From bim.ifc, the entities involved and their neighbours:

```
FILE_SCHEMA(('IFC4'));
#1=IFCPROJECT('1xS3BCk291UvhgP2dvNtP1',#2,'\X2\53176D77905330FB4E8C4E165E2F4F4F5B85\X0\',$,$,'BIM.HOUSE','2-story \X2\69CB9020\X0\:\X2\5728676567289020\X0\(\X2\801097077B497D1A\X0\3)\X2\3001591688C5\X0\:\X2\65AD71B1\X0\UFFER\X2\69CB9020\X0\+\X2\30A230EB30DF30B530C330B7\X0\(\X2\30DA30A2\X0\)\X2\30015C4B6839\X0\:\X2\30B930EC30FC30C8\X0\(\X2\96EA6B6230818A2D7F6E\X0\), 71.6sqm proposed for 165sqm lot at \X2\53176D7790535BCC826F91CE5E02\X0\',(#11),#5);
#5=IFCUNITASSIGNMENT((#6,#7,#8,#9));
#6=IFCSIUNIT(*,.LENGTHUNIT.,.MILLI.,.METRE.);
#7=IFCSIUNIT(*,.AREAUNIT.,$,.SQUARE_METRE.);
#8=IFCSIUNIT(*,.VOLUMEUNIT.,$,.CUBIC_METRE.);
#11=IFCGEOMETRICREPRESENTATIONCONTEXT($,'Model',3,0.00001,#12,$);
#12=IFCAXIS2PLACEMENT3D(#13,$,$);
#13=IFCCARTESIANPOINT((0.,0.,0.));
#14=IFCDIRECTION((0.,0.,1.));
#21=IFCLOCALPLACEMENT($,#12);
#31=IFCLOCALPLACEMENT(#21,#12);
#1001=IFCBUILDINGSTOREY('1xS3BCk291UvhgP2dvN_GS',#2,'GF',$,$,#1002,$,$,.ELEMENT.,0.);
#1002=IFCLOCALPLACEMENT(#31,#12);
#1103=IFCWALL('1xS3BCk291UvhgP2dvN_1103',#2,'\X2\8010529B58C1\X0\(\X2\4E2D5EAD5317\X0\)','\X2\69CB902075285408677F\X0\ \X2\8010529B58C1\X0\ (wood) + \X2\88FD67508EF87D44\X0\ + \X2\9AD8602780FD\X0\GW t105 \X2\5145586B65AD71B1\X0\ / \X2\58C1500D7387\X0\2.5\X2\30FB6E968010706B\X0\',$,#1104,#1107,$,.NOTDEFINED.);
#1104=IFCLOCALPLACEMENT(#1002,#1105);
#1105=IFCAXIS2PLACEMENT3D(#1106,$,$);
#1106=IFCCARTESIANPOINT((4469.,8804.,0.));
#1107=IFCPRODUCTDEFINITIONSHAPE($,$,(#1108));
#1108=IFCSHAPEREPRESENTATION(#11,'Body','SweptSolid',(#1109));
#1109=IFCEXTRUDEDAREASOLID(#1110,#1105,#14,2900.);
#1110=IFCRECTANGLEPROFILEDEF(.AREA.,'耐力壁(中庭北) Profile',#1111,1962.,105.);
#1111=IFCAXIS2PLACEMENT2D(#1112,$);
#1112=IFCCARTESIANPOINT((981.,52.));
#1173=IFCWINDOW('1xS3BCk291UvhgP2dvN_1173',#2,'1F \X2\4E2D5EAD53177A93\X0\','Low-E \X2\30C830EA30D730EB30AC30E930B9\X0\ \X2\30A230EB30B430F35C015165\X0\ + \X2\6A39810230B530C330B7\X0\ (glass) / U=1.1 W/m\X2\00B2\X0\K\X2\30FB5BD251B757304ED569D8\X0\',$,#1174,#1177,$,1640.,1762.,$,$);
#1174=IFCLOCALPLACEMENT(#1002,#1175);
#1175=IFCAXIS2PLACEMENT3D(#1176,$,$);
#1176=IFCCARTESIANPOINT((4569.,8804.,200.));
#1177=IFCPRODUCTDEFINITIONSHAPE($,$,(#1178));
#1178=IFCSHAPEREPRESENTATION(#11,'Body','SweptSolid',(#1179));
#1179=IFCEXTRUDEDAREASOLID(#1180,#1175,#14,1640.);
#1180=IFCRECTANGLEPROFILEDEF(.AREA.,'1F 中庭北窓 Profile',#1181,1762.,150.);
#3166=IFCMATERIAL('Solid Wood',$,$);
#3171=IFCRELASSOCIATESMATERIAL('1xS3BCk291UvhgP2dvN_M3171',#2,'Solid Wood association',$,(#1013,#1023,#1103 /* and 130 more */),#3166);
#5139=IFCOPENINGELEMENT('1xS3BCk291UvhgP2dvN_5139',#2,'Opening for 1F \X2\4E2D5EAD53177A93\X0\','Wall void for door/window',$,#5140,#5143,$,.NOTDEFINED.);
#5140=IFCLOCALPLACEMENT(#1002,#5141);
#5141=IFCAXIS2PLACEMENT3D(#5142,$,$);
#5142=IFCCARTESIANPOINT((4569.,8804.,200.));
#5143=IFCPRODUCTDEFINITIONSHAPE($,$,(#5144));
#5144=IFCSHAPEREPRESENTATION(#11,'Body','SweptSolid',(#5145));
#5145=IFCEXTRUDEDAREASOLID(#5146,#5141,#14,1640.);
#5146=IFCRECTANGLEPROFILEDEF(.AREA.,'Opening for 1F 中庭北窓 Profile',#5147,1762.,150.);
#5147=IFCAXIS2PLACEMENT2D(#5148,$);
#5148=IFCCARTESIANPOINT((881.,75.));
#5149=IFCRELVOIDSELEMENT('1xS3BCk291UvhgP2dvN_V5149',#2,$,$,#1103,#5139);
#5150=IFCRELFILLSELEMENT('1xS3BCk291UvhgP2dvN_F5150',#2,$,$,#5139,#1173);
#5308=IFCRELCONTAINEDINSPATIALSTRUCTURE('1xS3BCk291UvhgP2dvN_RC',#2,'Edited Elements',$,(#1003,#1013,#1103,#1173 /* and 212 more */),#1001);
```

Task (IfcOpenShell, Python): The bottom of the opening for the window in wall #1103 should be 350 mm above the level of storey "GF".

```python
import numpy as np
import ifcopenshell
import ifcopenshell.api.geometry
import ifcopenshell.geom
import ifcopenshell.util.element
import ifcopenshell.util.placement
import ifcopenshell.util.shape
import ifcopenshell.util.unit

model = ifcopenshell.open("bim.ifc")
unit_scale = ifcopenshell.util.unit.calculate_unit_scale(model)

window = model.by_id(1173)
opening = window.FillsVoids[0].RelatingOpeningElement
storey = ifcopenshell.util.element.get_container(window, ifc_class="IfcBuildingStorey")
level = ifcopenshell.util.placement.get_local_placement(storey.ObjectPlacement)[2, 3]

# The opening's origin need not be at the sill, so measure its lowest point.
shape = ifcopenshell.geom.create_shape(ifcopenshell.geom.settings(), opening)
bottom = ifcopenshell.util.shape.get_shape_bottom_elevation(shape, shape.geometry) / unit_scale
dz = level + 0.35 / unit_scale - bottom

shift = np.array([0.0, 0.0, dz])
# The window is not placed relative to its opening, so move both.
for product in (opening, window):
    matrix = ifcopenshell.util.placement.get_local_placement(product.ObjectPlacement)
    matrix[:3, 3] += shift
    ifcopenshell.api.geometry.edit_object_placement(model, product=product, matrix=matrix, is_si=False)

print(f"moved by {dz * unit_scale:+.3f} m")

model.write("bim_edited.ifc")
```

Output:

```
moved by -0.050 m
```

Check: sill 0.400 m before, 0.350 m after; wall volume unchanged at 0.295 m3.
